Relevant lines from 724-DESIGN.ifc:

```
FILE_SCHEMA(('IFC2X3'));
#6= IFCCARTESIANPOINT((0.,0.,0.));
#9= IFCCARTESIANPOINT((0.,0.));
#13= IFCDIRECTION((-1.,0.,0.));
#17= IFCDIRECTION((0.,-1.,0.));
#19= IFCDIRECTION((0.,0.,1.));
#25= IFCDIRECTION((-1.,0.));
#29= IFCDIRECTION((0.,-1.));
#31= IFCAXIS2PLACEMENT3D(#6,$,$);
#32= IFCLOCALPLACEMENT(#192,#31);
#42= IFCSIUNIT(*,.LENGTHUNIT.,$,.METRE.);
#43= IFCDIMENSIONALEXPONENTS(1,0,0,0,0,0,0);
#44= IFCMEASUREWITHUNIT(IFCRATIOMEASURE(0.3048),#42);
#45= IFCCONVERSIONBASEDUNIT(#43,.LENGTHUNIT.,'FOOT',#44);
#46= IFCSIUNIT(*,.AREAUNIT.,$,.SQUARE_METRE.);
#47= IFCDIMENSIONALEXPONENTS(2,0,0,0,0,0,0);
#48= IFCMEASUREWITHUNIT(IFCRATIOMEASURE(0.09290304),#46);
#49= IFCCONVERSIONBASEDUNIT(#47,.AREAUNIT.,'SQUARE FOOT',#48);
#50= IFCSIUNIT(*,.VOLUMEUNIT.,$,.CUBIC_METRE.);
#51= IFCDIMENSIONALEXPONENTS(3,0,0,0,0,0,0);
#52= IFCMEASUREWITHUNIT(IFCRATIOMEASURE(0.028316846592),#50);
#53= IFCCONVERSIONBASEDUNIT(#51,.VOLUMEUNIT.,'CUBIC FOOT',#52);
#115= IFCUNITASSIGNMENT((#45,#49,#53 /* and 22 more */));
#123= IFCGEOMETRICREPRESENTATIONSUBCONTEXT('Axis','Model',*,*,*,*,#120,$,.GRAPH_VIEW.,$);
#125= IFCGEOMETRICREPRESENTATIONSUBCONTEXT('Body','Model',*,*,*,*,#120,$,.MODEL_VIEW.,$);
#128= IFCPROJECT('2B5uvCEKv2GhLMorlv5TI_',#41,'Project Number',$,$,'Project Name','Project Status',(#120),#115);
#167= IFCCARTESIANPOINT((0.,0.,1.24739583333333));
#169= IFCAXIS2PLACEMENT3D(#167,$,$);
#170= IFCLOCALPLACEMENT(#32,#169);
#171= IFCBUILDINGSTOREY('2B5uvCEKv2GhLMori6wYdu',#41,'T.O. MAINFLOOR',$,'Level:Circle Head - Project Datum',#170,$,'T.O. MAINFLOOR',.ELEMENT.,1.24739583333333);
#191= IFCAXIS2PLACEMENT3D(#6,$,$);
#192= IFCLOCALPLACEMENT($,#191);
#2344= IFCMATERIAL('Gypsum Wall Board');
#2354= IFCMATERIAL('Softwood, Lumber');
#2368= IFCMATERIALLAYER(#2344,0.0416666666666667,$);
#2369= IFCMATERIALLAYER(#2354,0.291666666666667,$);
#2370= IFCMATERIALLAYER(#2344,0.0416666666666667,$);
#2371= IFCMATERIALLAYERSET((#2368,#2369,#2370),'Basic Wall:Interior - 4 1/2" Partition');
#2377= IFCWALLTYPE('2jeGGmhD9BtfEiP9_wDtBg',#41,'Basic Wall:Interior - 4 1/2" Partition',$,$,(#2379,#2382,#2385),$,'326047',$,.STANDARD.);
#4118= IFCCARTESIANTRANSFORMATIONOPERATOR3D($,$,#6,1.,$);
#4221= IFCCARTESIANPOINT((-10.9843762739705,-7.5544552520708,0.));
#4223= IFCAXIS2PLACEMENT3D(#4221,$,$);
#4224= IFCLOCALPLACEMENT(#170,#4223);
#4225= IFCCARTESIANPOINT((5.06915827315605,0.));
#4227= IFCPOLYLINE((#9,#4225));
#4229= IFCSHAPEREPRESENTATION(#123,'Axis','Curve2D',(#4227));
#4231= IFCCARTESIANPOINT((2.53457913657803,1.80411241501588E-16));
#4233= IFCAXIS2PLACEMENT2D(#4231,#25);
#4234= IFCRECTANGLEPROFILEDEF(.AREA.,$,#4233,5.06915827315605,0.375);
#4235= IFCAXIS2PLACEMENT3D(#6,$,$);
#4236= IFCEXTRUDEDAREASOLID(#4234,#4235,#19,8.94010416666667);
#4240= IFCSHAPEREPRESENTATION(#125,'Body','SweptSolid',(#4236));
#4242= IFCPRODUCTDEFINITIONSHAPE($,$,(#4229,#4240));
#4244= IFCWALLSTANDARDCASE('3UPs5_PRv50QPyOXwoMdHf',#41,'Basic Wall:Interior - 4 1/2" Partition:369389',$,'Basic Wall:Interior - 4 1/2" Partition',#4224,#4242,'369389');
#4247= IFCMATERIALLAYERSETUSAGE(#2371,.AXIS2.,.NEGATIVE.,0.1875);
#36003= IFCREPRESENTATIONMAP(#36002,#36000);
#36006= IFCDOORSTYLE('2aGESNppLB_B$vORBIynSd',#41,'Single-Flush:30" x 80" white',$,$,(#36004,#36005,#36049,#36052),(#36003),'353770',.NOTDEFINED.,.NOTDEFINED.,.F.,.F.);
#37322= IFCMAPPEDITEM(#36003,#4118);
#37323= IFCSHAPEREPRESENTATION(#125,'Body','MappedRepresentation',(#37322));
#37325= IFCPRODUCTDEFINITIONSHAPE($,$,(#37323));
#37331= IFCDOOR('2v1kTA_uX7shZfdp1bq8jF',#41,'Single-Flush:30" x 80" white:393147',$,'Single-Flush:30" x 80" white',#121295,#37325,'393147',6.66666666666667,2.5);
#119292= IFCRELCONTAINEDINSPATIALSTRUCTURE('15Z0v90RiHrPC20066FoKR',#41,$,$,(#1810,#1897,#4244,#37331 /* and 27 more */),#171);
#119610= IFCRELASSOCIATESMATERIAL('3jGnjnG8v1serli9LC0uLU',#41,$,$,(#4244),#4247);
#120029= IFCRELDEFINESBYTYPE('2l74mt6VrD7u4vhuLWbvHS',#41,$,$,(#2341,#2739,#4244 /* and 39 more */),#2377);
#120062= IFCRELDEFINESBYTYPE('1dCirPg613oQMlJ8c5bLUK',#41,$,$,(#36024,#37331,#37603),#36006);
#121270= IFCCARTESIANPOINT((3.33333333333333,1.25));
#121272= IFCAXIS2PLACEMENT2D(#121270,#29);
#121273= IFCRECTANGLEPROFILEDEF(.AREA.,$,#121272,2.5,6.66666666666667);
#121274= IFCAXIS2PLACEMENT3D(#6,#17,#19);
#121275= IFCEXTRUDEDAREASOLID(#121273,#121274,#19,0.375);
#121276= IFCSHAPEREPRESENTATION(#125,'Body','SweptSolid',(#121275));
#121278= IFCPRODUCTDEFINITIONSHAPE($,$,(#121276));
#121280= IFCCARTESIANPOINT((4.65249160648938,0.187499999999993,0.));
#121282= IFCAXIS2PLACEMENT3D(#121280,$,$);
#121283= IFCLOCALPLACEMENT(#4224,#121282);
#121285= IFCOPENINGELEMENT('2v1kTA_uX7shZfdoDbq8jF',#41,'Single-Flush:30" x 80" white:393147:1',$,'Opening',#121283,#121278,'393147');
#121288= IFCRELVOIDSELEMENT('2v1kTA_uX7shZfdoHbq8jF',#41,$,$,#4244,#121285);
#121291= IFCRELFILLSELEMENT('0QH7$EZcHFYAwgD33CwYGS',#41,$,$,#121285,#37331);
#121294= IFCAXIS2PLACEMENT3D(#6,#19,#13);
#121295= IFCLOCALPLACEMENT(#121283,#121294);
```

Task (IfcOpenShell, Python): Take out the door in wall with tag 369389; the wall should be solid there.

```python
import ifcopenshell
import ifcopenshell.api.feature
import ifcopenshell.api.root
import ifcopenshell.geom
import ifcopenshell.util.shape

model = ifcopenshell.open("724-DESIGN.ifc")
settings = ifcopenshell.geom.settings()


def volume(element):
    """Net volume in cubic metres, openings subtracted."""
    shape = ifcopenshell.geom.create_shape(settings, element)
    return ifcopenshell.util.shape.get_volume(shape.geometry)


door = model.by_guid("2v1kTA_uX7shZfdp1bq8jF")
opening = door.FillsVoids[0].RelatingOpeningElement
wall = opening.VoidsElements[0].RelatingBuildingElement
before = volume(wall)

ifcopenshell.api.root.remove_product(model, product=door)
ifcopenshell.api.feature.remove_feature(model, feature=opening)

after = volume(wall)

print(f"wall volume {before:.3f} -> {after:.3f} m3")

model.write("724-DESIGN_edited.ifc")
```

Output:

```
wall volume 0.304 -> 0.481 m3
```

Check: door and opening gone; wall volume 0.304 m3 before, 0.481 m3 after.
